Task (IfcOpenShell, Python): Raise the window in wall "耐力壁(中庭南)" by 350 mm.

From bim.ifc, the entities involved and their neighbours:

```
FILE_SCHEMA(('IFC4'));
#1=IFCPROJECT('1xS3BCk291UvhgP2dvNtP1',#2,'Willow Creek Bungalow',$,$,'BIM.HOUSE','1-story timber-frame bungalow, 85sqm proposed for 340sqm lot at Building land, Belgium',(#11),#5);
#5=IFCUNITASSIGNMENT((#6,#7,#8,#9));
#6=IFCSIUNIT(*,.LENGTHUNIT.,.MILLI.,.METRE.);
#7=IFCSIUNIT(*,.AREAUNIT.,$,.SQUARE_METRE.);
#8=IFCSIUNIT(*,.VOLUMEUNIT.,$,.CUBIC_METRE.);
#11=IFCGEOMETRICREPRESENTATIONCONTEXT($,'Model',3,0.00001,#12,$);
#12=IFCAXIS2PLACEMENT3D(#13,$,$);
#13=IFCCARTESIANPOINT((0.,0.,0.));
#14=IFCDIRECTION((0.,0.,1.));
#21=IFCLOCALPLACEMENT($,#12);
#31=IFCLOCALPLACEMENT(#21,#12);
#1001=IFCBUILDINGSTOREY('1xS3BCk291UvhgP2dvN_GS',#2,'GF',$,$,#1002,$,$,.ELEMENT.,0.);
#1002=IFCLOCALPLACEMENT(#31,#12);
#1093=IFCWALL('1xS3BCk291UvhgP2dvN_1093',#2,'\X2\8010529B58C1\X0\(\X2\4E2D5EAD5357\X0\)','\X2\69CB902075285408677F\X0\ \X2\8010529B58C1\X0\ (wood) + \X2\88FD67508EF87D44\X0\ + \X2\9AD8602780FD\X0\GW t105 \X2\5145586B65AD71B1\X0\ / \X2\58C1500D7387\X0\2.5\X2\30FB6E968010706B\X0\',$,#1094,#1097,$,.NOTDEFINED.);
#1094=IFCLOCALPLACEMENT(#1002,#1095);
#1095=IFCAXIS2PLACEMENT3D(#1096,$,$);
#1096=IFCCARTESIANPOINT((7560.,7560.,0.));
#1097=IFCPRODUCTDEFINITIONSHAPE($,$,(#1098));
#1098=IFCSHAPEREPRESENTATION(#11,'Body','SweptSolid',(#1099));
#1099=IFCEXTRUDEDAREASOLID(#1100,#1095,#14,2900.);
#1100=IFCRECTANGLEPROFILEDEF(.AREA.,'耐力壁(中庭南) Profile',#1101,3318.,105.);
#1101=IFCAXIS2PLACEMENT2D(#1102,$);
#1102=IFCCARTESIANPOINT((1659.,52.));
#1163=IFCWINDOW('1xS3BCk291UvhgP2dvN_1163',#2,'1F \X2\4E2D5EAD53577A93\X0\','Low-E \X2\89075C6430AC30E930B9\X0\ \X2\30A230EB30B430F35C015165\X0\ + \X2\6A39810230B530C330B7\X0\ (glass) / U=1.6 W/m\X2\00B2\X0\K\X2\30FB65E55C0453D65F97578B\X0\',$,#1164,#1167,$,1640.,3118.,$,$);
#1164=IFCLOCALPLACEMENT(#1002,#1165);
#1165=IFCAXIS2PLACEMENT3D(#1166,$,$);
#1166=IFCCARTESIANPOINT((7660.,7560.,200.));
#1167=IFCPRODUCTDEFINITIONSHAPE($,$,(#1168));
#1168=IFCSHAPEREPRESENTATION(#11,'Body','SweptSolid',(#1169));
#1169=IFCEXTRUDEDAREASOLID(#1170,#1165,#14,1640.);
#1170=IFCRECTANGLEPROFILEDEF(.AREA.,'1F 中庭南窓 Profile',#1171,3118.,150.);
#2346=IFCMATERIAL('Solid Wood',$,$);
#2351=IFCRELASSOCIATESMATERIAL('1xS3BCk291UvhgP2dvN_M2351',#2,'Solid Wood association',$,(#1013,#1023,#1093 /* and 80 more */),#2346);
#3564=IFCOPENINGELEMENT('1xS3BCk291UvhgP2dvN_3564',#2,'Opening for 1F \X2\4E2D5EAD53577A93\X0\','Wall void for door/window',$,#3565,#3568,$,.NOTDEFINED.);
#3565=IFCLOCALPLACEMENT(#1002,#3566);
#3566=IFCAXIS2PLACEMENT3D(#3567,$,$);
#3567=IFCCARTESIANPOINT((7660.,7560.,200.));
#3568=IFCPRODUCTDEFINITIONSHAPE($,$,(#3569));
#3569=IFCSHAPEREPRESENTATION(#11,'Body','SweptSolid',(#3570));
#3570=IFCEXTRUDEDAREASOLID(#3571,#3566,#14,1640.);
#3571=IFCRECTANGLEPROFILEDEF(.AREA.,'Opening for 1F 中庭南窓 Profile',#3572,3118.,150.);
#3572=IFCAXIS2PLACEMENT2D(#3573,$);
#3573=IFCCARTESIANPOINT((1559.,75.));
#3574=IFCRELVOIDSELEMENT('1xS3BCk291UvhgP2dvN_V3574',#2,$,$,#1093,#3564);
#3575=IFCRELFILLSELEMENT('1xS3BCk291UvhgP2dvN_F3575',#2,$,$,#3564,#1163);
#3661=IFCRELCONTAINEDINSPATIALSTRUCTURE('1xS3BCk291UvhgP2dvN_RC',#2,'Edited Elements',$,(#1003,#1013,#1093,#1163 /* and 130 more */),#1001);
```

```python
import numpy as np
import ifcopenshell
import ifcopenshell.api.geometry
import ifcopenshell.util.placement
import ifcopenshell.util.unit

model = ifcopenshell.open("bim.ifc")
unit_scale = ifcopenshell.util.unit.calculate_unit_scale(model)

window = model.by_id(1163)
opening = window.FillsVoids[0].RelatingOpeningElement
dz = 350.0

shift = np.array([0.0, 0.0, dz])
# The window is not placed relative to its opening, so move both.
for product in (opening, window):
    matrix = ifcopenshell.util.placement.get_local_placement(product.ObjectPlacement)
    matrix[:3, 3] += shift
    ifcopenshell.api.geometry.edit_object_placement(model, product=product, matrix=matrix, is_si=False)

print(f"moved by {dz * unit_scale:+.3f} m")

model.write("bim_updated.ifc")
```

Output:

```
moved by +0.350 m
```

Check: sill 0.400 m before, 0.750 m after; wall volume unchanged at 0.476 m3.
